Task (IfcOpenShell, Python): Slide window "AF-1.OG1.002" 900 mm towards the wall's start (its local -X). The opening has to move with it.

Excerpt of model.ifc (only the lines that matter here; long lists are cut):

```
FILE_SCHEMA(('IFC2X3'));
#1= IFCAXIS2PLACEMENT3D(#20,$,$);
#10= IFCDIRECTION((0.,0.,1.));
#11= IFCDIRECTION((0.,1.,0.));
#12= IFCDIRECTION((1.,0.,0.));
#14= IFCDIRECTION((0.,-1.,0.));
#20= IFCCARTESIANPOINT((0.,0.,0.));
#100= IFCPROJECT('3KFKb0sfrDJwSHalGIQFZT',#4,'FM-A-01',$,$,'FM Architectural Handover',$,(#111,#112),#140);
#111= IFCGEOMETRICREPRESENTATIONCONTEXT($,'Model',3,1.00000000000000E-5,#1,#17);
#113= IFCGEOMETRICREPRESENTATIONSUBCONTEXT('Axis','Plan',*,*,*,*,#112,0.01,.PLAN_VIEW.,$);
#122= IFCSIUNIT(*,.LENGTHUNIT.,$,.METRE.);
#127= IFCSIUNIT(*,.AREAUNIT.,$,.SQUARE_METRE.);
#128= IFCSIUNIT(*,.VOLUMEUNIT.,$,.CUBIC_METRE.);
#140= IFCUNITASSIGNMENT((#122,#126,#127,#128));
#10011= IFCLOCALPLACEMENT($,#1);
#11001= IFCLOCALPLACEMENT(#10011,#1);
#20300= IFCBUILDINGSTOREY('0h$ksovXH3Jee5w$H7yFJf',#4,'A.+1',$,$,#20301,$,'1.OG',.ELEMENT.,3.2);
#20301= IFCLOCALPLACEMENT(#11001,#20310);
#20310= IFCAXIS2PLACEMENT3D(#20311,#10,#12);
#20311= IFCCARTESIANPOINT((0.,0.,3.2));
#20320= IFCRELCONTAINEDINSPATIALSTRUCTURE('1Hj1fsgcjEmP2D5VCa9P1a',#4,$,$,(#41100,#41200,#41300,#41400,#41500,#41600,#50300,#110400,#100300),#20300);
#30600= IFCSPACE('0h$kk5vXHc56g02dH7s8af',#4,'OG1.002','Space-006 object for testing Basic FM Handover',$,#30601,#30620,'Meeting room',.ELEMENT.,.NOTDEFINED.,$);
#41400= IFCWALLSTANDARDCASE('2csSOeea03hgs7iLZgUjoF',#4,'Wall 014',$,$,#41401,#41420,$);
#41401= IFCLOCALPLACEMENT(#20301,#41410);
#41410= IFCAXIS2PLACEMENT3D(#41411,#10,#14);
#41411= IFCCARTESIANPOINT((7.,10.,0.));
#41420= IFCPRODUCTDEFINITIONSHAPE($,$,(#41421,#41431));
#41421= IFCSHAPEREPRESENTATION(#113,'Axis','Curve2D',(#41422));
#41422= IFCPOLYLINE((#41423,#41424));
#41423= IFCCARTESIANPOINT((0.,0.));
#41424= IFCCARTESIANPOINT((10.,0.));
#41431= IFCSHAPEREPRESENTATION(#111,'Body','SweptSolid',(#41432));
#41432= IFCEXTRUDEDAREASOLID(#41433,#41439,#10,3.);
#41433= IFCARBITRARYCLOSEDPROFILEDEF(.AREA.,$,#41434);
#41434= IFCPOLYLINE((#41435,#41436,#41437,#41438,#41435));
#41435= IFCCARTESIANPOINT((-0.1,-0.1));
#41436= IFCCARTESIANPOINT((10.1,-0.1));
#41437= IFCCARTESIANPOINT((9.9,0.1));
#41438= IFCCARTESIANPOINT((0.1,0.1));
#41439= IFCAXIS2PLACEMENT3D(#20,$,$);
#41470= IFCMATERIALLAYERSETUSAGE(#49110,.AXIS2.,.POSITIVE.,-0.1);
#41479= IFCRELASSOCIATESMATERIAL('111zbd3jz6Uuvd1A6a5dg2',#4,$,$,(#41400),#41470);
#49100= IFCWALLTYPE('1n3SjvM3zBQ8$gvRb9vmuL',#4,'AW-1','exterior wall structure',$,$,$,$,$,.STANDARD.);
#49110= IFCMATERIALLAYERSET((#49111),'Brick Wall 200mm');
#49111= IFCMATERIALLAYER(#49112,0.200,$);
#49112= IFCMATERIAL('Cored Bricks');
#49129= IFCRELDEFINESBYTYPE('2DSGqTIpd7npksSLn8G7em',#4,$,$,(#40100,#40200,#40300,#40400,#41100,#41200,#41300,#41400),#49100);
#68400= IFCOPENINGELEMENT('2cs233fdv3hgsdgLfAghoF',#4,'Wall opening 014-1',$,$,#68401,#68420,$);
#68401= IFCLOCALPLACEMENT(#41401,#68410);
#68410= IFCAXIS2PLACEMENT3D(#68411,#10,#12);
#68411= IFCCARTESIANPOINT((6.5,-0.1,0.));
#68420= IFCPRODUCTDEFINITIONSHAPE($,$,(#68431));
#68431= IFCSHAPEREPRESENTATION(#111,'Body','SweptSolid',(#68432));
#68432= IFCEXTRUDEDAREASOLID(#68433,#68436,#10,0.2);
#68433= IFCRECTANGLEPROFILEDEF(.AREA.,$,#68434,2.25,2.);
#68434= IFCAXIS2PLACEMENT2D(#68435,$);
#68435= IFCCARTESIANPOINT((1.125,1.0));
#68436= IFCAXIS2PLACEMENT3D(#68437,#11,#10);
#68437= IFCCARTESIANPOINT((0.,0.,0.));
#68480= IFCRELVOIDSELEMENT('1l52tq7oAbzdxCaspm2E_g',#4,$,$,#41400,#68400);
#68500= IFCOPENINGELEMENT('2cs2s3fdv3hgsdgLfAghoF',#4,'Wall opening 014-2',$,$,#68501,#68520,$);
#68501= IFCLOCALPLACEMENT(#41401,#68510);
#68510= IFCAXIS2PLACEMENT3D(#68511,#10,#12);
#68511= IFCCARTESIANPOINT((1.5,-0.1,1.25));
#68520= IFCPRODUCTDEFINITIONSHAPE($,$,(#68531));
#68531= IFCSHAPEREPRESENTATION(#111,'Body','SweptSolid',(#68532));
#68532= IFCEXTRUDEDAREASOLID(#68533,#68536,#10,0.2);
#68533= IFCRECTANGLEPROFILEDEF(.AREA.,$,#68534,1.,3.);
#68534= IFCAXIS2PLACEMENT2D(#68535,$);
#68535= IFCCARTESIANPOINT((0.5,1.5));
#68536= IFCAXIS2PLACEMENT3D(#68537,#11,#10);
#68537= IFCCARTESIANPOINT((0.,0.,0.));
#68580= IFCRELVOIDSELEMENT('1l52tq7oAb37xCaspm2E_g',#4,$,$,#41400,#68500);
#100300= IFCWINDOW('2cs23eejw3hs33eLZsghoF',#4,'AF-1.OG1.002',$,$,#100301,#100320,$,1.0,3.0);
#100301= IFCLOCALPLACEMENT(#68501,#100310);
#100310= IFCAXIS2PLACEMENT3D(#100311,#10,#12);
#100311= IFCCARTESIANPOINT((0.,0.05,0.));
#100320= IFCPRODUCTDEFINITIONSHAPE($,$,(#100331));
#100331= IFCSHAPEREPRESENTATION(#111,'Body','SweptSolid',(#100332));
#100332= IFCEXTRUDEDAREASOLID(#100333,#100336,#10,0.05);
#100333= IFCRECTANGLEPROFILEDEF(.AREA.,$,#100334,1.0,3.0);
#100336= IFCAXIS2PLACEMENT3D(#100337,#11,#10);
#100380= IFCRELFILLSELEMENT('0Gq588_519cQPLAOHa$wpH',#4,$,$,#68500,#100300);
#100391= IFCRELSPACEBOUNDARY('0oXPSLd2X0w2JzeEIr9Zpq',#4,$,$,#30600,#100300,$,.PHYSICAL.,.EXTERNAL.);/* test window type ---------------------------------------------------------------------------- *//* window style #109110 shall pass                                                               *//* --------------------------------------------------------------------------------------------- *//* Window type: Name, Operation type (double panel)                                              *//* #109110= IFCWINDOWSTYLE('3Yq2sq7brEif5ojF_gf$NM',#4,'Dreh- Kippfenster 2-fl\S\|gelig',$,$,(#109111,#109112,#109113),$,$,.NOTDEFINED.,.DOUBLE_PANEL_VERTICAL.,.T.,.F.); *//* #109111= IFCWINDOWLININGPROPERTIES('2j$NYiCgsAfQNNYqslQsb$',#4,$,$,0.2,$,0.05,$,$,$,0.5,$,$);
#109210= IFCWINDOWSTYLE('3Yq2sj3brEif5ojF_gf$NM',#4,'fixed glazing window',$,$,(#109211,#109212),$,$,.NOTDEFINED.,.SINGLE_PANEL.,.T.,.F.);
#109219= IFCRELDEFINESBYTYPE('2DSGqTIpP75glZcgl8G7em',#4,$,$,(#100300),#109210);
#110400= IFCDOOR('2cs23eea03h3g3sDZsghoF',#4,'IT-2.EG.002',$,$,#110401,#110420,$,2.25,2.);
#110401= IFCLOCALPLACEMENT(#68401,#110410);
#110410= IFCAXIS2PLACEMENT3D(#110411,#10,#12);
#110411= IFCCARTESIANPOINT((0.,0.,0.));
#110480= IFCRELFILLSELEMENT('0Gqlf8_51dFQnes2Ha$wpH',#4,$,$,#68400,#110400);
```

```python
import ifcopenshell
import ifcopenshell.api.geometry
import ifcopenshell.util.placement

model = ifcopenshell.open("model.ifc")

window = model.by_id(100300)
opening = window.FillsVoids[0].RelatingOpeningElement
wall = opening.VoidsElements[0].RelatingBuildingElement

wall_matrix = ifcopenshell.util.placement.get_local_placement(wall.ObjectPlacement)
shift = wall_matrix[:3, 0] * -0.9
before = ifcopenshell.util.placement.get_local_placement(window.ObjectPlacement)[:3, 3].copy()

# The window is placed relative to its opening, so it follows when the opening moves.
matrix = ifcopenshell.util.placement.get_local_placement(opening.ObjectPlacement)
matrix[:3, 3] += shift
ifcopenshell.api.geometry.edit_object_placement(
    model, product=opening, matrix=matrix, is_si=False, should_transform_children=True
)

after = ifcopenshell.util.placement.get_local_placement(window.ObjectPlacement)[:3, 3]
print("window moved by", (after - before).round(3) + 0.0)

model.write("model-out.ifc")
```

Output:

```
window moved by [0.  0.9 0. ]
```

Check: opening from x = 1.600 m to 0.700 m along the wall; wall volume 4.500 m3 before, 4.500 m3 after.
